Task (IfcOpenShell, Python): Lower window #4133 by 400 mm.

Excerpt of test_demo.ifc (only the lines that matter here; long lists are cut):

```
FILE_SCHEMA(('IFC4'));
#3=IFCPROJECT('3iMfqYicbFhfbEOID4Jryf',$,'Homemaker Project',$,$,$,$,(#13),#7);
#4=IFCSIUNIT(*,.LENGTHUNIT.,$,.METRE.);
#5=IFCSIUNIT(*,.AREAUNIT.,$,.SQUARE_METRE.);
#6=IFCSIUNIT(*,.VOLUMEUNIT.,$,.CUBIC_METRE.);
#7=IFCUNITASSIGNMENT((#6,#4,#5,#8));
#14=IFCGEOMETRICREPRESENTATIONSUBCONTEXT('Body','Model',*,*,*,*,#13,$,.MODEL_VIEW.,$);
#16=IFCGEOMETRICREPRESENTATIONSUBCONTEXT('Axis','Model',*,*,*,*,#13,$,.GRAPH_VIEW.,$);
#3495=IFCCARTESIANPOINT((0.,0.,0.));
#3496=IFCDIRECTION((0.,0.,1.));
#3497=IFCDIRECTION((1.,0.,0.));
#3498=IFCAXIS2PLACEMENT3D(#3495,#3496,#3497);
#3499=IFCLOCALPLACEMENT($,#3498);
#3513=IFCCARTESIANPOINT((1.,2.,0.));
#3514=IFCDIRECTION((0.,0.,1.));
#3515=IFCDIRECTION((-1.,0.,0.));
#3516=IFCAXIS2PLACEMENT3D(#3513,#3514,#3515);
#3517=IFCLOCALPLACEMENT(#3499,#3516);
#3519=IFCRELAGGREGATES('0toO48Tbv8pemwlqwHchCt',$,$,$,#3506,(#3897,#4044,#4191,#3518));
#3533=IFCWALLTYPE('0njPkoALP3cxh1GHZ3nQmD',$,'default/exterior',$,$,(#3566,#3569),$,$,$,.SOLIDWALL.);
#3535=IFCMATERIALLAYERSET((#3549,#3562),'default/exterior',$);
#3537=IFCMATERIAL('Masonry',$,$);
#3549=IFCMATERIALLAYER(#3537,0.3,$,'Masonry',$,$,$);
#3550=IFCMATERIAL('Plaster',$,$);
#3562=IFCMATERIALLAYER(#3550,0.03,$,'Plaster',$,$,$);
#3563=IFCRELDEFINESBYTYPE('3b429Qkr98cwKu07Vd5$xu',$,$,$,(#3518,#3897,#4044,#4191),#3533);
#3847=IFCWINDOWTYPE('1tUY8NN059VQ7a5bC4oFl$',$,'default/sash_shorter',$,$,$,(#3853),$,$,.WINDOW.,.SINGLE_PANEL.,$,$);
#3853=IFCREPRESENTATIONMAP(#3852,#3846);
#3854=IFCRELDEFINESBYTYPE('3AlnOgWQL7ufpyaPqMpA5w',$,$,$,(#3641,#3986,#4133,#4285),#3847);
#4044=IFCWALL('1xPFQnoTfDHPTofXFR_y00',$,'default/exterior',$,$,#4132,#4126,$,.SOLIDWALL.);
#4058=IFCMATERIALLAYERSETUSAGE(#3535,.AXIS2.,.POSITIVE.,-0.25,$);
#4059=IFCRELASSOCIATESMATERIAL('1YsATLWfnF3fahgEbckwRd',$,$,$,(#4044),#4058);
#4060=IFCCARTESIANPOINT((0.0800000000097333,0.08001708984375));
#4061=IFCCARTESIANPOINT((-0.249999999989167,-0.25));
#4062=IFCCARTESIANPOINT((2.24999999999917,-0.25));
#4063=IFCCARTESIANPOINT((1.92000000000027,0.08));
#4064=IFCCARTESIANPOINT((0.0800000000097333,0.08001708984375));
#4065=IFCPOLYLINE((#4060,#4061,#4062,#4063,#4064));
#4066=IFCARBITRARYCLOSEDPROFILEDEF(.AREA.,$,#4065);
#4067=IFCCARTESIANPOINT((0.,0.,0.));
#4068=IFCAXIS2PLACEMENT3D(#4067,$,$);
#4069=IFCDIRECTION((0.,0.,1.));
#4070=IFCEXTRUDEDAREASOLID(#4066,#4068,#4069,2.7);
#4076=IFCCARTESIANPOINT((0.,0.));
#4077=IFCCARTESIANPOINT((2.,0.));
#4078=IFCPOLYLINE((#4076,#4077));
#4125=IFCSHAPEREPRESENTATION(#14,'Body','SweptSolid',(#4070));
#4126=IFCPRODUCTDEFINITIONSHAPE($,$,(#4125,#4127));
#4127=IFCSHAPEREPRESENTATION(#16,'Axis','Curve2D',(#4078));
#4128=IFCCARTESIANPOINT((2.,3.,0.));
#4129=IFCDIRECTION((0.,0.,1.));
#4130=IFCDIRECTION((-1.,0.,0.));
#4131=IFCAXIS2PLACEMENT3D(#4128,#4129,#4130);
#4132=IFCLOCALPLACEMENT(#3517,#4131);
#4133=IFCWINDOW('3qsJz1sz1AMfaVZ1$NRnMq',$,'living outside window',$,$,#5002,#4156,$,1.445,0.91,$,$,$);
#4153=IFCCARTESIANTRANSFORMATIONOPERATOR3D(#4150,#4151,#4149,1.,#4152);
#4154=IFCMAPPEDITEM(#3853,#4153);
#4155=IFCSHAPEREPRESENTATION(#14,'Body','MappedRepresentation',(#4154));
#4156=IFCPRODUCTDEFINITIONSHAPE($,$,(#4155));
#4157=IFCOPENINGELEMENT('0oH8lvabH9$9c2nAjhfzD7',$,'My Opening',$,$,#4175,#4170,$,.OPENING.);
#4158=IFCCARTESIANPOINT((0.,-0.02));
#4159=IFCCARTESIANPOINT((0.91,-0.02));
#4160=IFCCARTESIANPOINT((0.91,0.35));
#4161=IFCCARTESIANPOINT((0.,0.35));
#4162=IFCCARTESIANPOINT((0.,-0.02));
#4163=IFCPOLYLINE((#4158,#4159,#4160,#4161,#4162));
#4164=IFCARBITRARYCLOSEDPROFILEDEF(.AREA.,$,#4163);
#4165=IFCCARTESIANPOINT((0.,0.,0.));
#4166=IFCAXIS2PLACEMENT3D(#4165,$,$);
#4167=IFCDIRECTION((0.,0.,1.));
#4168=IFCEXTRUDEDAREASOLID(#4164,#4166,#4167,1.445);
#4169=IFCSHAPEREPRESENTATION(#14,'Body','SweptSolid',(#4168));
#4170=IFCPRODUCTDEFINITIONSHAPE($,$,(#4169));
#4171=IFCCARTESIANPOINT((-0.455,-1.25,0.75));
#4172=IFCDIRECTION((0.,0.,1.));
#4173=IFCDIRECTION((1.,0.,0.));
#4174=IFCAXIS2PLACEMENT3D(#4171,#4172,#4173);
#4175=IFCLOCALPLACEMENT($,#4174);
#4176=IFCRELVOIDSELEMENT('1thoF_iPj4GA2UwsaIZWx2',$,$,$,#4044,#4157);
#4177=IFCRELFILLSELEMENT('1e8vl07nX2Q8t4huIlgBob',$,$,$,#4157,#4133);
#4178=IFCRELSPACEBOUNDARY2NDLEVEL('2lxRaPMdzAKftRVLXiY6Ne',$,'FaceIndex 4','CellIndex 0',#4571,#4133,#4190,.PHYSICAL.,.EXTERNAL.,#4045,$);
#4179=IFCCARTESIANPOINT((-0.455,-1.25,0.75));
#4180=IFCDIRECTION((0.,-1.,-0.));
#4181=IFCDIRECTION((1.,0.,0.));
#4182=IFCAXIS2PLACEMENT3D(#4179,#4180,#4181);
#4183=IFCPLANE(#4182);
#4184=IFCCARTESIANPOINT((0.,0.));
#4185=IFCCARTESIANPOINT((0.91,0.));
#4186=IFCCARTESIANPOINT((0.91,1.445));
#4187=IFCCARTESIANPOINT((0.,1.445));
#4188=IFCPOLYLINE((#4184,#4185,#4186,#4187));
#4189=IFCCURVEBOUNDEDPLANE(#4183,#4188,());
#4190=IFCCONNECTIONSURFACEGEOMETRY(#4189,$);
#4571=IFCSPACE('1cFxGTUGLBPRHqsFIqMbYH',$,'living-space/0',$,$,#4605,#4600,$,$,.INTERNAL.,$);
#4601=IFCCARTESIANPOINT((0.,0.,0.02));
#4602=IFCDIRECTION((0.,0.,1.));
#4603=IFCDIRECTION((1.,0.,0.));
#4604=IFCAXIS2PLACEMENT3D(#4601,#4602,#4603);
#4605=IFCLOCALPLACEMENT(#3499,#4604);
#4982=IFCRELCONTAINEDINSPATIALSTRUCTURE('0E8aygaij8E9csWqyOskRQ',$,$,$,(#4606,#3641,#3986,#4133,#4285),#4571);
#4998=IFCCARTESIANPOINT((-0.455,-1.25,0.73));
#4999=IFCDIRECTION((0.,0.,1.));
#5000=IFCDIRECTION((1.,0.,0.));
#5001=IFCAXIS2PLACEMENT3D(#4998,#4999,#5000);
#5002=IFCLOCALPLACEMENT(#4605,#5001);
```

```python
import numpy as np
import ifcopenshell
import ifcopenshell.api.geometry
import ifcopenshell.util.placement
import ifcopenshell.util.unit

model = ifcopenshell.open("test_demo.ifc")
unit_scale = ifcopenshell.util.unit.calculate_unit_scale(model)

window = model.by_guid("3qsJz1sz1AMfaVZ1$NRnMq")
opening = window.FillsVoids[0].RelatingOpeningElement
dz = -0.4

shift = np.array([0.0, 0.0, dz])
# The window is not placed relative to its opening, so move both.
for product in (opening, window):
    matrix = ifcopenshell.util.placement.get_local_placement(product.ObjectPlacement)
    matrix[:3, 3] += shift
    ifcopenshell.api.geometry.edit_object_placement(model, product=product, matrix=matrix, is_si=False)

# Space boundary surfaces are stored in each space's coordinates; move them too.
for rel in window.ProvidesBoundaries:
    if not rel.ConnectionGeometry:
        continue
    surface = rel.ConnectionGeometry.SurfaceOnRelatingElement.BasisSurface
    space_matrix = ifcopenshell.util.placement.get_local_placement(rel.RelatingSpace.ObjectPlacement)
    point = np.array(surface.Position.Location.Coordinates) + space_matrix[:3, :3].T @ shift
    surface.Position = model.createIfcAxis2Placement3D(
        model.createIfcCartesianPoint(point.tolist()), surface.Position.Axis, surface.Position.RefDirection
    )

print(f"moved by {dz * unit_scale:+.3f} m")

model.write("test_demo_rev.ifc")
```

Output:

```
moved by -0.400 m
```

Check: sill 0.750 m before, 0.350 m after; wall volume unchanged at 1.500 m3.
